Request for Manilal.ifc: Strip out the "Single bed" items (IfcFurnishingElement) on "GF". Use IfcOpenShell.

First a look at what the model holds.

```python
import ifcopenshell
import ifcopenshell.util.element

model = ifcopenshell.open("Manilal.ifc")
print(model.schema)
storey = next(s for s in model.by_type("IfcBuildingStorey") if s.Name == "GF")
furniture = [e for e in ifcopenshell.util.element.get_decomposition(storey) if e.is_a("IfcFurnishingElement")]
seen = {}
for e in furniture:
    element_type = ifcopenshell.util.element.get_type(e)
    name = element_type.Name if element_type not in (None, e) else None
    seen[name] = seen.get(name, 0) + 1
for name, count in sorted(seen.items(), key=str):
    print(count, "x", name)
```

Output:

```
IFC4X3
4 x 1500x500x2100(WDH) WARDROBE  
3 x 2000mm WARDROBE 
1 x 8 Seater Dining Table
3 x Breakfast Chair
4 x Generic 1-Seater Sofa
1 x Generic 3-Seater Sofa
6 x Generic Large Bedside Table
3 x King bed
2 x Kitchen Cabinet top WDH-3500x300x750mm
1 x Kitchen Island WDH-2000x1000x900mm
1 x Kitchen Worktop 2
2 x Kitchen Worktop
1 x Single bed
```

```python
import ifcopenshell
import ifcopenshell.api.root
import ifcopenshell.util.element

model = ifcopenshell.open("Manilal.ifc")

storey = next(s for s in model.by_type("IfcBuildingStorey") if s.Name == "GF")
furniture = [e for e in ifcopenshell.util.element.get_decomposition(storey) if e.is_a("IfcFurnishingElement")]
targets = [e for e in furniture if (t := ifcopenshell.util.element.get_type(e)) not in (None, e) and t.Name == "Single bed"]

for e in targets:
    ifcopenshell.api.root.remove_product(model, product=e)
print(len(targets), "removed")

model.write("Manilal_updated.ifc")
```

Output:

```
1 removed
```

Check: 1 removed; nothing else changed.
